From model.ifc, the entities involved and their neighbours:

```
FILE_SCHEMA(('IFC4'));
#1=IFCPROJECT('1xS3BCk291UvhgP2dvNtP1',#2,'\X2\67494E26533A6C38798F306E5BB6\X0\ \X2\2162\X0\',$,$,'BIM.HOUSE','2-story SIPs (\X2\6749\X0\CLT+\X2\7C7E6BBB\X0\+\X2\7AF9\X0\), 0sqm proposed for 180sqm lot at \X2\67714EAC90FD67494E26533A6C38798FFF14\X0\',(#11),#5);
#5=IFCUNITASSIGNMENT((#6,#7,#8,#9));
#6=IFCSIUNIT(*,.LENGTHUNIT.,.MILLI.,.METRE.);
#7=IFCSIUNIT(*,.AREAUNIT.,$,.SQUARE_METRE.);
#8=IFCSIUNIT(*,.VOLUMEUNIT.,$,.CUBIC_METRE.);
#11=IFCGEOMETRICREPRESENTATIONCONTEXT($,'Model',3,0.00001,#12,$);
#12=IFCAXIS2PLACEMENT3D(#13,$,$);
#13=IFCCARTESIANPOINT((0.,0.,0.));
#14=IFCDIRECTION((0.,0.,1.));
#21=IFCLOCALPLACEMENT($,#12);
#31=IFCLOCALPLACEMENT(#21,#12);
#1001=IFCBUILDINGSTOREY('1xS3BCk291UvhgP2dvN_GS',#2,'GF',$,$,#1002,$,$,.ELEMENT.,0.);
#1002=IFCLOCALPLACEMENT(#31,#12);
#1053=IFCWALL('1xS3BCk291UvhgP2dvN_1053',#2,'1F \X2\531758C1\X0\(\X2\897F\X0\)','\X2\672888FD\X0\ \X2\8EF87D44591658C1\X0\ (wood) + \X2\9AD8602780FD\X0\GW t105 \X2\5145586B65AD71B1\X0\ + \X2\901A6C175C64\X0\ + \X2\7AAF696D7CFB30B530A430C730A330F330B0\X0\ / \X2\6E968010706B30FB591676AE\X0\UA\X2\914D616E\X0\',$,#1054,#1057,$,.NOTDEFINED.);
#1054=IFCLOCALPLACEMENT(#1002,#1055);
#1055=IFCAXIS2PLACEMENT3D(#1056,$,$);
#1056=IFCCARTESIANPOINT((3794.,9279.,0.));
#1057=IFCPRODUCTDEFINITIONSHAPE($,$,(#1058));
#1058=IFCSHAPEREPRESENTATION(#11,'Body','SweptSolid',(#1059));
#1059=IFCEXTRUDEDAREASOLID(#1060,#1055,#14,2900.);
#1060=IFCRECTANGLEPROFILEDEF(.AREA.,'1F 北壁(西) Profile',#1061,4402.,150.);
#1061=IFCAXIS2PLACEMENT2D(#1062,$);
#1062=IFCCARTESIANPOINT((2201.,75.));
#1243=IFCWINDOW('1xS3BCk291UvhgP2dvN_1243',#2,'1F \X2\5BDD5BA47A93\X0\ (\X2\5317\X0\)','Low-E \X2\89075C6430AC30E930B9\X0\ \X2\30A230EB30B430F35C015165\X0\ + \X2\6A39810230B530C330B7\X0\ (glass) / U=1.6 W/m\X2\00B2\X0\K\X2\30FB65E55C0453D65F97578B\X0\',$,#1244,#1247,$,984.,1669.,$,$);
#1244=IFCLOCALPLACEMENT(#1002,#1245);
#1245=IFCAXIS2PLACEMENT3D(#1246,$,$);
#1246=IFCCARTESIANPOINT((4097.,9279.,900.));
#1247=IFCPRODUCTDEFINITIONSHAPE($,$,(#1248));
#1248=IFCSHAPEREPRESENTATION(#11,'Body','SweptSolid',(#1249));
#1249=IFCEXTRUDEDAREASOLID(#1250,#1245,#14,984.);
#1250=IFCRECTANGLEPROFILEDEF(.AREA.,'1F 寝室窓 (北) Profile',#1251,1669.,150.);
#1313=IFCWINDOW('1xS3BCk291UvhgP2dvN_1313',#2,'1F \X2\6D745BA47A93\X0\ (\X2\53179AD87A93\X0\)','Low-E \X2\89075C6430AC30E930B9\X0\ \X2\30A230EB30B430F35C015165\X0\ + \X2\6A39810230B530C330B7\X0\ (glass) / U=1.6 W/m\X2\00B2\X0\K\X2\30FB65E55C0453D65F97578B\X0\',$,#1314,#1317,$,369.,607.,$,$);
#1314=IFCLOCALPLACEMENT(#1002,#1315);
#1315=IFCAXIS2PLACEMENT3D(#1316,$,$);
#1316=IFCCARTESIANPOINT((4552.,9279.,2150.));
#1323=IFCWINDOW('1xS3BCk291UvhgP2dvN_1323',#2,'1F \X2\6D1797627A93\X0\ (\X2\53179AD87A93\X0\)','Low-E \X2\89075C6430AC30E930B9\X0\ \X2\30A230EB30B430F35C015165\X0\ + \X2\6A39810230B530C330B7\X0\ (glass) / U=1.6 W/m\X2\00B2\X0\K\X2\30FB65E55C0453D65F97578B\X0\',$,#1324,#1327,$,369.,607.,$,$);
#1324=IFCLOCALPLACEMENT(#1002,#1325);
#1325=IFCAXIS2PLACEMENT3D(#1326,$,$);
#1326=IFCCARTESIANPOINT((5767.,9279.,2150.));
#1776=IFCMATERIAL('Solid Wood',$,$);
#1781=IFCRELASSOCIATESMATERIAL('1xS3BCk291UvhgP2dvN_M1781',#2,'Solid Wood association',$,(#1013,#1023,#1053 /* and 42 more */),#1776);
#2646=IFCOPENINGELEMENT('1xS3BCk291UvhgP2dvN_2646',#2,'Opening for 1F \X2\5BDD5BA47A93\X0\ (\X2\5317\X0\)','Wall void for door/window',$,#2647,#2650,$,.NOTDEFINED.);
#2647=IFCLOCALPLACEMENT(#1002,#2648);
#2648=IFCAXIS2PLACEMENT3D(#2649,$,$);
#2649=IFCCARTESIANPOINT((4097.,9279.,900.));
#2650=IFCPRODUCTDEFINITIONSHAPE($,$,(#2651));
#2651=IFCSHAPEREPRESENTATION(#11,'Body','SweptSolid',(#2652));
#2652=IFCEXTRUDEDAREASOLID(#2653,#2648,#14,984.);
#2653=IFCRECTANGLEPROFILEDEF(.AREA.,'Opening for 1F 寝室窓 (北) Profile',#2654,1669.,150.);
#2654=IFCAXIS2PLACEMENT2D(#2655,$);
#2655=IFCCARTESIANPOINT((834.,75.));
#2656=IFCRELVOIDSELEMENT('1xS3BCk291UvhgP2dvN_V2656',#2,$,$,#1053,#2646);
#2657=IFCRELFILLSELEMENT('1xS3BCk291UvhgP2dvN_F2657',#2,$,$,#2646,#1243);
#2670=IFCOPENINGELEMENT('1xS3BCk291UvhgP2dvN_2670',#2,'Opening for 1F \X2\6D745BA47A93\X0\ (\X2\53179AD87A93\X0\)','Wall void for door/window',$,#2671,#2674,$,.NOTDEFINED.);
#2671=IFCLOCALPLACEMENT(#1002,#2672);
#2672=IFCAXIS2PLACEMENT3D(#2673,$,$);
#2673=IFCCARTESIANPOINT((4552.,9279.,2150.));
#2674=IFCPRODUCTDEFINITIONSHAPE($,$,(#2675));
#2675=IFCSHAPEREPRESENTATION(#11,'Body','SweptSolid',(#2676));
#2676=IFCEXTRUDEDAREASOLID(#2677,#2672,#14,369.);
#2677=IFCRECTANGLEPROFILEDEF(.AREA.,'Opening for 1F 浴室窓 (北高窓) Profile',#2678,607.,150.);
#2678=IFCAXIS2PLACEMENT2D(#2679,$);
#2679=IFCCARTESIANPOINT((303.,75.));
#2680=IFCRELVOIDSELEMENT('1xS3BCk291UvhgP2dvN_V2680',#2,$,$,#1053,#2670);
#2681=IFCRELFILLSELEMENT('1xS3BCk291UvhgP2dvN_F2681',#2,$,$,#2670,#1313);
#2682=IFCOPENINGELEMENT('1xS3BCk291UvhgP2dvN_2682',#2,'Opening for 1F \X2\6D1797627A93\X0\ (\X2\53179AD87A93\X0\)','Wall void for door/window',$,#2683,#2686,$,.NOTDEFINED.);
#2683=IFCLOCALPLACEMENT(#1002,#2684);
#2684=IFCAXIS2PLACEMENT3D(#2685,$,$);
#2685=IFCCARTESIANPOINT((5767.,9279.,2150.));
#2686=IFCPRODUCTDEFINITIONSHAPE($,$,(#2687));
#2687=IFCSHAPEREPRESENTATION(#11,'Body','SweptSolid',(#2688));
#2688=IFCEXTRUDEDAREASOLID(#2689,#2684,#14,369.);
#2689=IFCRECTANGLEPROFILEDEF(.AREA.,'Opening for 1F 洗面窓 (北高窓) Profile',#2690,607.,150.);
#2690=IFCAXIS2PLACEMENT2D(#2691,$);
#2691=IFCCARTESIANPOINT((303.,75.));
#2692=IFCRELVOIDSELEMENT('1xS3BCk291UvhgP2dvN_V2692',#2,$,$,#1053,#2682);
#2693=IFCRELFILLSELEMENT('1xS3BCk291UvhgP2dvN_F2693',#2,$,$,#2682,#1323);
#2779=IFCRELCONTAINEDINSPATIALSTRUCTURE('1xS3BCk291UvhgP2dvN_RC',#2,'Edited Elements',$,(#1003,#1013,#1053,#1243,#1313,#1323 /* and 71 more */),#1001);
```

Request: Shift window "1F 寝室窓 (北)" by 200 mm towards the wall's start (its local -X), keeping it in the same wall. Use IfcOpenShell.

```python
import ifcopenshell
import ifcopenshell.api.geometry
import ifcopenshell.util.placement
import ifcopenshell.util.unit

model = ifcopenshell.open("model.ifc")
unit_scale = ifcopenshell.util.unit.calculate_unit_scale(model)

window = model.by_id(1243)
opening = window.FillsVoids[0].RelatingOpeningElement
wall = opening.VoidsElements[0].RelatingBuildingElement

wall_matrix = ifcopenshell.util.placement.get_local_placement(wall.ObjectPlacement)
shift = wall_matrix[:3, 0] * -0.2 / unit_scale
before = ifcopenshell.util.placement.get_local_placement(window.ObjectPlacement)[:3, 3].copy()

# The window is not placed relative to its opening, so move both.
for product in (opening, window):
    matrix = ifcopenshell.util.placement.get_local_placement(product.ObjectPlacement)
    matrix[:3, 3] += shift
    ifcopenshell.api.geometry.edit_object_placement(model, product=product, matrix=matrix, is_si=False)

after = ifcopenshell.util.placement.get_local_placement(window.ObjectPlacement)[:3, 3]
print("window moved by", (after - before).round(3) + 0.0)

model.write("model_edited.ifc")
```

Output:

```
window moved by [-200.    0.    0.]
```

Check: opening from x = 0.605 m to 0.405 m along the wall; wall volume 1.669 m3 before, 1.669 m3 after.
